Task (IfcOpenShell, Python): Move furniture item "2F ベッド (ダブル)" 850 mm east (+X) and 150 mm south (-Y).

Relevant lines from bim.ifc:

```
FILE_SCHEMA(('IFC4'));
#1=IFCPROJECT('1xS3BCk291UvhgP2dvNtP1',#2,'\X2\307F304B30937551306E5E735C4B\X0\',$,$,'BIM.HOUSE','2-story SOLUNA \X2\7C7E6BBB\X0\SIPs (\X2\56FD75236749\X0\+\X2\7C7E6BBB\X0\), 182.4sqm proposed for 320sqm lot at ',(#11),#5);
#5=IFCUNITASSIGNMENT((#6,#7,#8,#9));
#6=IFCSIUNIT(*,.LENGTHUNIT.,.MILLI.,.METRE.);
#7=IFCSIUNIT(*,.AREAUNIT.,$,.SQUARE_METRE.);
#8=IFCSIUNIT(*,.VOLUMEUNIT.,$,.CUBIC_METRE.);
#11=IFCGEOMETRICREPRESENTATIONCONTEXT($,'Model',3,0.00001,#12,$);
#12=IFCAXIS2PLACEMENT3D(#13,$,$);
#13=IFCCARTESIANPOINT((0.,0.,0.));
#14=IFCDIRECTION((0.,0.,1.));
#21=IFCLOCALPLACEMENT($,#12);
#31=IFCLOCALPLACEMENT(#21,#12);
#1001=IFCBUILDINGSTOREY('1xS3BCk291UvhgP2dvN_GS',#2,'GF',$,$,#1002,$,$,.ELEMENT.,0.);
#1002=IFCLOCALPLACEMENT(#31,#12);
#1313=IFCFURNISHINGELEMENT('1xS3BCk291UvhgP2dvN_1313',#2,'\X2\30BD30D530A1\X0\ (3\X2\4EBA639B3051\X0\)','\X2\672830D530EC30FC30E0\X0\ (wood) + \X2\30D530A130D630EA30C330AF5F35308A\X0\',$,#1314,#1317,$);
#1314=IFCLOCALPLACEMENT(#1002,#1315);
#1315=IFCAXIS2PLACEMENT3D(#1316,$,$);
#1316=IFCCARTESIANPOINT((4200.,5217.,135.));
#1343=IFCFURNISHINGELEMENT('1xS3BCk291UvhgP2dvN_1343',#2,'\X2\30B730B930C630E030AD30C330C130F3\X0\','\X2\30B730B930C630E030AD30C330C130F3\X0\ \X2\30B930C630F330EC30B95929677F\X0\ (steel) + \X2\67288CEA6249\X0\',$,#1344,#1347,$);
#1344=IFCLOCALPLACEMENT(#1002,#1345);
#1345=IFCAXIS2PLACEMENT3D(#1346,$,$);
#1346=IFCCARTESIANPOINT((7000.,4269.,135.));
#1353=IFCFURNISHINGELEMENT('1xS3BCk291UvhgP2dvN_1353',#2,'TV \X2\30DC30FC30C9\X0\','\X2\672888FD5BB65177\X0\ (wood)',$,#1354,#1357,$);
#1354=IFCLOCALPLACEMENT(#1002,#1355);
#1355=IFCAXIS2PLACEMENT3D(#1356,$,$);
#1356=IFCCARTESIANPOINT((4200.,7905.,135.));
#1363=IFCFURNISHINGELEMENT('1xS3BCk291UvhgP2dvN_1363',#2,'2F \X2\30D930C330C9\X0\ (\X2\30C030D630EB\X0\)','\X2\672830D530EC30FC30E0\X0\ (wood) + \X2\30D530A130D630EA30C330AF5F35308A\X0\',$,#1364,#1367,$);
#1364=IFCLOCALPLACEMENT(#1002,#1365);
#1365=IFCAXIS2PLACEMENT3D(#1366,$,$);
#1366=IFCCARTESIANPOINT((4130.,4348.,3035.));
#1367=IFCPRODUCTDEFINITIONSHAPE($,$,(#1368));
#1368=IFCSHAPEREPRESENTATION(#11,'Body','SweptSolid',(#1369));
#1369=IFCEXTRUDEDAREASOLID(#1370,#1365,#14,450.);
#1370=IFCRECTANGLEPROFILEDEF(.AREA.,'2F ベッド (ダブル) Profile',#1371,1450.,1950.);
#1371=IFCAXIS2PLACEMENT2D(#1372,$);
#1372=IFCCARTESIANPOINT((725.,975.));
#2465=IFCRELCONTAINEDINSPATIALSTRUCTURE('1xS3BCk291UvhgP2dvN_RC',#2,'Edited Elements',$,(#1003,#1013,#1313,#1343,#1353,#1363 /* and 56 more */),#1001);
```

```python
import ifcopenshell
import ifcopenshell.api.geometry
import ifcopenshell.util.placement

model = ifcopenshell.open("bim.ifc")

item = model.by_id(1363)
matrix = ifcopenshell.util.placement.get_local_placement(item.ObjectPlacement)
matrix[0, 3] += 850.0
matrix[1, 3] -= 150.0
ifcopenshell.api.geometry.edit_object_placement(model, product=item, matrix=matrix, is_si=False)

print(ifcopenshell.util.placement.get_local_placement(item.ObjectPlacement).round(3) + 0.0)

model.write("bim_v2.ifc")
```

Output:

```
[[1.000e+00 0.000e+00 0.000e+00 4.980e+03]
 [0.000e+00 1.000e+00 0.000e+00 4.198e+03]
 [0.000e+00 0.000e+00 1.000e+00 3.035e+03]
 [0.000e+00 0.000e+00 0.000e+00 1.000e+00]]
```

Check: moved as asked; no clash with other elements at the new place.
